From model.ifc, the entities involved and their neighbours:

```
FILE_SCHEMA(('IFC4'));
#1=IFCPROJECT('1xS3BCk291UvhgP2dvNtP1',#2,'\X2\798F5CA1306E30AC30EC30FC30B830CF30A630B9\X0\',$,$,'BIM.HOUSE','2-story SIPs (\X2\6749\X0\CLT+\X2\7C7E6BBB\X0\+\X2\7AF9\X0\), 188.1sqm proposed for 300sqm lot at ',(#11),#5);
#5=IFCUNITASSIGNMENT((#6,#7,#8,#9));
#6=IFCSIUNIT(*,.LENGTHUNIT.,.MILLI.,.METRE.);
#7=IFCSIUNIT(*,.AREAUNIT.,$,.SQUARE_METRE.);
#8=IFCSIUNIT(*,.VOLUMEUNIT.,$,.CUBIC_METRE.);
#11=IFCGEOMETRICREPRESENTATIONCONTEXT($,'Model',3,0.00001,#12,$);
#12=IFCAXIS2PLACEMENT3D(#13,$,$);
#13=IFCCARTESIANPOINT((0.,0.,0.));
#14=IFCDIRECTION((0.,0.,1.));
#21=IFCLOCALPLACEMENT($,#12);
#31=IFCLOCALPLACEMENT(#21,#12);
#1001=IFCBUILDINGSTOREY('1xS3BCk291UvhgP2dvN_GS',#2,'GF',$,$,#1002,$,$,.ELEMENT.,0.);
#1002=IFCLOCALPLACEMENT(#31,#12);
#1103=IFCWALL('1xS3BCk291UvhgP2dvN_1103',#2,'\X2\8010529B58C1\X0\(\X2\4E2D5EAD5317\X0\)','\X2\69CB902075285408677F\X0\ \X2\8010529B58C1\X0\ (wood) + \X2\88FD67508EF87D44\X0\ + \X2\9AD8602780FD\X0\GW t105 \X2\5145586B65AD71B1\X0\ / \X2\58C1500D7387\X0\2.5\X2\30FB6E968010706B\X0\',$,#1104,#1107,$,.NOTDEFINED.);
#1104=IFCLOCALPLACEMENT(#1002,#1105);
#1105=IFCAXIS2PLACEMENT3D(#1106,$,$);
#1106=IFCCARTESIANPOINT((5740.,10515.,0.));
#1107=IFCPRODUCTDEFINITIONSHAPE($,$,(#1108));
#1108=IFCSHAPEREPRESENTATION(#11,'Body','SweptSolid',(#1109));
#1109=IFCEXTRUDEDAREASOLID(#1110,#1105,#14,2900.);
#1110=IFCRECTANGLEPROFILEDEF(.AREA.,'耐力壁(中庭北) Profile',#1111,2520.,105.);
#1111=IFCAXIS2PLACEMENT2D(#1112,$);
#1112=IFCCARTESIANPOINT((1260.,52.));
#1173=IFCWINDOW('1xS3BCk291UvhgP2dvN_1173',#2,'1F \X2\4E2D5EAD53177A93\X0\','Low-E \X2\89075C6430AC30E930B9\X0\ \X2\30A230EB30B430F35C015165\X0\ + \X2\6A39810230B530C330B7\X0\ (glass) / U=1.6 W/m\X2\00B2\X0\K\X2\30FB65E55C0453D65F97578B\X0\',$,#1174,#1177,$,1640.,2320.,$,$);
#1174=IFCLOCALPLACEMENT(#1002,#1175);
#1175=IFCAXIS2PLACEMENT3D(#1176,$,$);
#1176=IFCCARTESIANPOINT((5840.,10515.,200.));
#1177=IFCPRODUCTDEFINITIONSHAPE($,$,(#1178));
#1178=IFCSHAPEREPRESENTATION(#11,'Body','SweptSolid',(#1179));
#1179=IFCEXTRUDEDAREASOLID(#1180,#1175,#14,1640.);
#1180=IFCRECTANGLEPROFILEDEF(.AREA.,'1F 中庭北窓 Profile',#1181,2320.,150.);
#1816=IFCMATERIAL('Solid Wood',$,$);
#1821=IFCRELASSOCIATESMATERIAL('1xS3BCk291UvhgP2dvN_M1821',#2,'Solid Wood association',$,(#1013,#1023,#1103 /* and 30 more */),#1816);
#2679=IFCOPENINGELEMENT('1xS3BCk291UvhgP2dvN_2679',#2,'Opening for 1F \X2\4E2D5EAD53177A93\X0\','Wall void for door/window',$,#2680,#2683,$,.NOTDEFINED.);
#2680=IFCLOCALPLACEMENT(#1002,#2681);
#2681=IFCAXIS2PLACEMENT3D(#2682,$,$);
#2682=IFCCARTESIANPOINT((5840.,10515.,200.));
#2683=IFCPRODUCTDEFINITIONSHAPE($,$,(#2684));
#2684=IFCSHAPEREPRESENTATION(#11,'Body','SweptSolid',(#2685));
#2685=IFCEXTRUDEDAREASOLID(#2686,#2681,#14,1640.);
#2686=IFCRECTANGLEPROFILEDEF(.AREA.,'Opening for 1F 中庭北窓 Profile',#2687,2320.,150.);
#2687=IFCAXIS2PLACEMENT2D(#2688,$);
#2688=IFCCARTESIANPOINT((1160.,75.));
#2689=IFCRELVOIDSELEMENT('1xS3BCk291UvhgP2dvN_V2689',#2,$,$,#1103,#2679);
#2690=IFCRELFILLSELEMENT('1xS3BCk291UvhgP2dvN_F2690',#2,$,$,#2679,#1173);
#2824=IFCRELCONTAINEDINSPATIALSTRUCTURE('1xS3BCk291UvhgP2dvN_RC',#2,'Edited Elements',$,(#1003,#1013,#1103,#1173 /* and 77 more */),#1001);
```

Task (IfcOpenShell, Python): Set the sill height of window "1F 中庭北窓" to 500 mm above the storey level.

```python
import numpy as np
import ifcopenshell
import ifcopenshell.api.geometry
import ifcopenshell.geom
import ifcopenshell.util.element
import ifcopenshell.util.placement
import ifcopenshell.util.shape
import ifcopenshell.util.unit

model = ifcopenshell.open("model.ifc")
unit_scale = ifcopenshell.util.unit.calculate_unit_scale(model)

window = model.by_guid("1xS3BCk291UvhgP2dvN_1173")
opening = window.FillsVoids[0].RelatingOpeningElement
storey = ifcopenshell.util.element.get_container(window, ifc_class="IfcBuildingStorey")
level = ifcopenshell.util.placement.get_local_placement(storey.ObjectPlacement)[2, 3]

# The opening's origin need not be at the sill, so measure its lowest point.
shape = ifcopenshell.geom.create_shape(ifcopenshell.geom.settings(), opening)
bottom = ifcopenshell.util.shape.get_shape_bottom_elevation(shape, shape.geometry) / unit_scale
dz = level + 0.5 / unit_scale - bottom

shift = np.array([0.0, 0.0, dz])
# The window is not placed relative to its opening, so move both.
for product in (opening, window):
    matrix = ifcopenshell.util.placement.get_local_placement(product.ObjectPlacement)
    matrix[:3, 3] += shift
    ifcopenshell.api.geometry.edit_object_placement(model, product=product, matrix=matrix, is_si=False)

print(f"moved by {dz * unit_scale:+.3f} m")

model.write("model_v2.ifc")
```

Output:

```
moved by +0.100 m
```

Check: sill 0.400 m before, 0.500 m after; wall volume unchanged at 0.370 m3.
